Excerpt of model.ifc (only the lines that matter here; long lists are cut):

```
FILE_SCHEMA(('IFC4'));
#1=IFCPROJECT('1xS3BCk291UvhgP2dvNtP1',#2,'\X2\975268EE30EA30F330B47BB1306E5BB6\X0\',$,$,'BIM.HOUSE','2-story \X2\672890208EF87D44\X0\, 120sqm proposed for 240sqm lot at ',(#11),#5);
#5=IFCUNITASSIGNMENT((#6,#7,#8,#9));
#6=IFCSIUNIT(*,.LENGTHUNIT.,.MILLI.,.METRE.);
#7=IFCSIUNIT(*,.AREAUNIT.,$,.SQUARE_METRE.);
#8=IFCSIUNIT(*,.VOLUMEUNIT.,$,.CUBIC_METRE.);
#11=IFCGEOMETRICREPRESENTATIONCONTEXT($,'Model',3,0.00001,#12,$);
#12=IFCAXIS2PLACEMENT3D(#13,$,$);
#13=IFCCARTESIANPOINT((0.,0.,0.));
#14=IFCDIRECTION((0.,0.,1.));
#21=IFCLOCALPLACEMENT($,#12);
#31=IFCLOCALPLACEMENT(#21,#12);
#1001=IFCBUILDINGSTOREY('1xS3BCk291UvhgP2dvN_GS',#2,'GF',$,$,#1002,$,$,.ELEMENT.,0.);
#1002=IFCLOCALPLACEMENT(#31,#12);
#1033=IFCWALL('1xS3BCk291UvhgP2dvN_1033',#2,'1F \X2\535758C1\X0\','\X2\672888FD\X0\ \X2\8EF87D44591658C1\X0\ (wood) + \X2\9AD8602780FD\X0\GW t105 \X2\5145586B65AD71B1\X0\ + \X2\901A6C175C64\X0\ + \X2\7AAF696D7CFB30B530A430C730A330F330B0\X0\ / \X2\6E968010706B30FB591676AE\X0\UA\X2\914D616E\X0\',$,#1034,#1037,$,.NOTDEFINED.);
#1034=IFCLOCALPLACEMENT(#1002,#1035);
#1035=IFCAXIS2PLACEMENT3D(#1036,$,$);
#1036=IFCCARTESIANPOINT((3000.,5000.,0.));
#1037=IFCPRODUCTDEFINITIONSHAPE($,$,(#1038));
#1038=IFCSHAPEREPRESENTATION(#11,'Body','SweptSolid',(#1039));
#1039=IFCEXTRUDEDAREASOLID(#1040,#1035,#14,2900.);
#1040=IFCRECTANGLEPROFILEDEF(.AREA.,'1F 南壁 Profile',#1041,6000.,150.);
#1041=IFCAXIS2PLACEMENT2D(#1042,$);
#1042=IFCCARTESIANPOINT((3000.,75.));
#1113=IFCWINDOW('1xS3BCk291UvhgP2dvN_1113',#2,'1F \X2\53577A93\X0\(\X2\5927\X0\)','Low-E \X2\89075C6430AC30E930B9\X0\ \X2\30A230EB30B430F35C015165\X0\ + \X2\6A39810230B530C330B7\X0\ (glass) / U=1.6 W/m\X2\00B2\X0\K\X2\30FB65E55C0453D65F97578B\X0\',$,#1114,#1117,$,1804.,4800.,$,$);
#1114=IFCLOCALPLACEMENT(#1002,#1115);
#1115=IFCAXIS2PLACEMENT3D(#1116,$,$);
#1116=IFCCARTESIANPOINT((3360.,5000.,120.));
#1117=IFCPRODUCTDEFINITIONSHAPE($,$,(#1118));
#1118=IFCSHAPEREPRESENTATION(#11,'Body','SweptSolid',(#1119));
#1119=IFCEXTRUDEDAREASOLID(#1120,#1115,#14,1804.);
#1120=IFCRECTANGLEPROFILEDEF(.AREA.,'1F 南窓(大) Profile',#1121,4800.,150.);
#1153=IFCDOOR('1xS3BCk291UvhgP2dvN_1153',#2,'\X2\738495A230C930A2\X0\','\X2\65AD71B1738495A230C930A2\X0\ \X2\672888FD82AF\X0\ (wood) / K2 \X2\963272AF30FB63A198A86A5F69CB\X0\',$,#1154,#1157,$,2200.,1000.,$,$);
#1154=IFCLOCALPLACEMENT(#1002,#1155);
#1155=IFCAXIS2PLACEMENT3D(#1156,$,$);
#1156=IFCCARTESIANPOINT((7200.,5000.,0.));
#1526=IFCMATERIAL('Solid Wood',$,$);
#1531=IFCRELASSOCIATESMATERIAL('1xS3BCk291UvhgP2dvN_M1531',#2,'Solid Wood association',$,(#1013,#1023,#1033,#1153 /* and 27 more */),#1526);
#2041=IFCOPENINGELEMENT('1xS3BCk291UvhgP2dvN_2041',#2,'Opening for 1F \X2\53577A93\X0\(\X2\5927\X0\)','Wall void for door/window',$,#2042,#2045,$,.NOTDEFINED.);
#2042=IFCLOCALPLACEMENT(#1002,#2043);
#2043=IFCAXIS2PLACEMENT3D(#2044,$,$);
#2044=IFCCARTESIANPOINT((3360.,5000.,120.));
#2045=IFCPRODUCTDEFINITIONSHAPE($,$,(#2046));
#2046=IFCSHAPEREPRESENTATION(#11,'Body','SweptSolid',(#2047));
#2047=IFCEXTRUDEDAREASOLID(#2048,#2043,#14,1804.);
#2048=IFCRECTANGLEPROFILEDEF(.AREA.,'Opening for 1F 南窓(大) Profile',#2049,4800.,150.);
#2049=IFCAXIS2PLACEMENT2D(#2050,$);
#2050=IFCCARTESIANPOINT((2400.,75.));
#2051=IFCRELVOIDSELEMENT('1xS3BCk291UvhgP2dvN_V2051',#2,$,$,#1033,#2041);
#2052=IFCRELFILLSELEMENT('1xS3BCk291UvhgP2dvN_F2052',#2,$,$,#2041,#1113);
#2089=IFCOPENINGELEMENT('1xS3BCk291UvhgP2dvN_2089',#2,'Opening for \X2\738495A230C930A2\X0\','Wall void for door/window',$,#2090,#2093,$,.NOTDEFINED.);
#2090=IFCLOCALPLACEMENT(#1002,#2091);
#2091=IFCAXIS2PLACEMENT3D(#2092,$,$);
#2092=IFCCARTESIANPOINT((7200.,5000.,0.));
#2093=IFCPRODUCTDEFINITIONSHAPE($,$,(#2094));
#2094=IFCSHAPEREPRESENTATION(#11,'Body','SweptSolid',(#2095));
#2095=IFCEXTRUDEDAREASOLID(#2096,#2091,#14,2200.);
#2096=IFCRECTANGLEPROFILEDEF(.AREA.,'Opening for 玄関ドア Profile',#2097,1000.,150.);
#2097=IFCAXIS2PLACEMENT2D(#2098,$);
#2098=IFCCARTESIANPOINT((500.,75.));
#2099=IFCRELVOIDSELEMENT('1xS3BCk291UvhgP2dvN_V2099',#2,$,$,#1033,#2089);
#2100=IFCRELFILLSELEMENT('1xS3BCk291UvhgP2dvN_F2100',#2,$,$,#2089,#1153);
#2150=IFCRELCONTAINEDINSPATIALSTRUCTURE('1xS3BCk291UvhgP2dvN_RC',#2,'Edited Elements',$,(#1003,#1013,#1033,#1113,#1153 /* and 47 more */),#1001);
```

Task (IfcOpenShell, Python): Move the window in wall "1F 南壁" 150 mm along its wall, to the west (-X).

```python
import ifcopenshell
import ifcopenshell.api.geometry
import ifcopenshell.util.placement
import ifcopenshell.util.unit

model = ifcopenshell.open("model.ifc")
unit_scale = ifcopenshell.util.unit.calculate_unit_scale(model)

window = model.by_id(1113)
opening = window.FillsVoids[0].RelatingOpeningElement
wall = opening.VoidsElements[0].RelatingBuildingElement

wall_matrix = ifcopenshell.util.placement.get_local_placement(wall.ObjectPlacement)
shift = wall_matrix[:3, 0] * -0.15 / unit_scale
before = ifcopenshell.util.placement.get_local_placement(window.ObjectPlacement)[:3, 3].copy()

# The window is not placed relative to its opening, so move both.
for product in (opening, window):
    matrix = ifcopenshell.util.placement.get_local_placement(product.ObjectPlacement)
    matrix[:3, 3] += shift
    ifcopenshell.api.geometry.edit_object_placement(model, product=product, matrix=matrix, is_si=False)

after = ifcopenshell.util.placement.get_local_placement(window.ObjectPlacement)[:3, 3]
print("window moved by", (after - before).round(3) + 0.0)

model.write("model-out.ifc")
```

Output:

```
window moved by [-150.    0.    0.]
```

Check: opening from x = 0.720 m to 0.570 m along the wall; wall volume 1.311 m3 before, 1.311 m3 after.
